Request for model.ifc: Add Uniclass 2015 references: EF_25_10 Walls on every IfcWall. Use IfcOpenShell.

First a look at what the model holds.

```python
import ifcopenshell

model = ifcopenshell.open("model.ifc")
print(model.schema)
print("classifications:", [c.Name for c in model.by_type("IfcClassification")])
for ifc_class in ("IfcDoor", "IfcRoof", "IfcStair", "IfcWall", "IfcWindow"):
    print(ifc_class, len(model.by_type(ifc_class)))
```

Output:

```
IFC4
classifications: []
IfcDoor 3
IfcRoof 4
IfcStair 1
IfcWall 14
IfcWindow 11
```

```python
import ifcopenshell
import ifcopenshell.api.classification

model = ifcopenshell.open("model.ifc")

system = ifcopenshell.api.classification.add_classification(model, classification="Uniclass 2015")

codes = {
    "IfcWall": ("EF_25_10", "Walls"),
}
for ifc_class, (code, name) in codes.items():
    products = model.by_type(ifc_class)
    ifcopenshell.api.classification.add_reference(
        model, products=products, classification=system, identification=code, name=name
    )
    print(code, len(products))

model.write("model_updated.ifc")
```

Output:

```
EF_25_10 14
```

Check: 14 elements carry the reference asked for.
